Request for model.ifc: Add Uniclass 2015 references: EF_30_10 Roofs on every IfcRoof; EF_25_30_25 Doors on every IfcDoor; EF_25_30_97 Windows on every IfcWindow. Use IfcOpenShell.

First a look at what the model holds.

```python
import ifcopenshell

model = ifcopenshell.open("model.ifc")
print(model.schema)
print("classifications:", [c.Name for c in model.by_type("IfcClassification")])
for ifc_class in ("IfcDoor", "IfcRoof", "IfcStair", "IfcWall", "IfcWindow"):
    print(ifc_class, len(model.by_type(ifc_class)))
```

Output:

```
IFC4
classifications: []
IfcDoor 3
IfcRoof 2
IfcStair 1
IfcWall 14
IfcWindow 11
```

```python
import ifcopenshell
import ifcopenshell.api.classification

model = ifcopenshell.open("model.ifc")

system = ifcopenshell.api.classification.add_classification(model, classification="Uniclass 2015")

codes = {
    "IfcRoof": ("EF_30_10", "Roofs"),
    "IfcDoor": ("EF_25_30_25", "Doors"),
    "IfcWindow": ("EF_25_30_97", "Windows"),
}
for ifc_class, (code, name) in codes.items():
    products = model.by_type(ifc_class)
    ifcopenshell.api.classification.add_reference(
        model, products=products, classification=system, identification=code, name=name
    )
    print(code, len(products))

model.write("model_edited.ifc")
```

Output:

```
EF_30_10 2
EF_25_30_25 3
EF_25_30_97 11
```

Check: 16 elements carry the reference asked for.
